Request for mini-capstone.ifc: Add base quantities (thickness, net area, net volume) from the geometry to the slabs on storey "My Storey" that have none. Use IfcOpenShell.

First a look at what the model holds.

```python
import ifcopenshell
import ifcopenshell.util.element
import ifcopenshell.util.unit

model = ifcopenshell.open("mini-capstone.ifc")
print(model.schema)
for unit_type in ("LENGTHUNIT", "AREAUNIT", "VOLUMEUNIT"):
    print(unit_type, ifcopenshell.util.unit.calculate_unit_scale(model, unit_type))
storey = next(s for s in model.by_type("IfcBuildingStorey") if s.Name == "My Storey")
slabs = [e for e in ifcopenshell.util.element.get_decomposition(storey) if e.is_a("IfcSlab")]
for e in sorted(slabs, key=lambda e: e.id()):
    print(e.id(), e.is_a(), e.Name, list(ifcopenshell.util.element.get_psets(e, qtos_only=True)), sep=" | ")
```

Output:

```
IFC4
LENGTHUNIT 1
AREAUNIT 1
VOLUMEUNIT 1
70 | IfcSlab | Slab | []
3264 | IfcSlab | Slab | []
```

```python
import ifcopenshell
import ifcopenshell.api.pset
import ifcopenshell.geom
import ifcopenshell.util.element
import ifcopenshell.util.shape
import ifcopenshell.util.unit

model = ifcopenshell.open("mini-capstone.ifc")
unit_scale = ifcopenshell.util.unit.calculate_unit_scale(model)
area_scale = ifcopenshell.util.unit.calculate_unit_scale(model, "AREAUNIT")
volume_scale = ifcopenshell.util.unit.calculate_unit_scale(model, "VOLUMEUNIT")
settings = ifcopenshell.geom.settings()

storey = next(s for s in model.by_type("IfcBuildingStorey") if s.Name == "My Storey")
slabs = [e for e in ifcopenshell.util.element.get_decomposition(storey) if e.is_a("IfcSlab")]

for e in sorted(slabs, key=lambda e: e.id()):
    if ifcopenshell.util.element.get_psets(e, qtos_only=True, should_inherit=False):
        continue
    # Geometry comes back in metres, in the element's own axes.
    shape = ifcopenshell.geom.create_shape(settings, e)
    values = {
        "Width": ifcopenshell.util.shape.get_z(shape.geometry) / unit_scale,
        "NetArea": ifcopenshell.util.shape.get_footprint_area(shape.geometry) / area_scale,
        "NetVolume": ifcopenshell.util.shape.get_volume(shape.geometry) / volume_scale,
    }
    qto = ifcopenshell.api.pset.add_qto(model, product=e, name="Qto_SlabBaseQuantities")
    ifcopenshell.api.pset.edit_qto(model, qto=qto, properties=values)
    print(e.id(), {k: round(v, 3) for k, v in values.items()})

model.write("mini-capstone_updated.ifc")
```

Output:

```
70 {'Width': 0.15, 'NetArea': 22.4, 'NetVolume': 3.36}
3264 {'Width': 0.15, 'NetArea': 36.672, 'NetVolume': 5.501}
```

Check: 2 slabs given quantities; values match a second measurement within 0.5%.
